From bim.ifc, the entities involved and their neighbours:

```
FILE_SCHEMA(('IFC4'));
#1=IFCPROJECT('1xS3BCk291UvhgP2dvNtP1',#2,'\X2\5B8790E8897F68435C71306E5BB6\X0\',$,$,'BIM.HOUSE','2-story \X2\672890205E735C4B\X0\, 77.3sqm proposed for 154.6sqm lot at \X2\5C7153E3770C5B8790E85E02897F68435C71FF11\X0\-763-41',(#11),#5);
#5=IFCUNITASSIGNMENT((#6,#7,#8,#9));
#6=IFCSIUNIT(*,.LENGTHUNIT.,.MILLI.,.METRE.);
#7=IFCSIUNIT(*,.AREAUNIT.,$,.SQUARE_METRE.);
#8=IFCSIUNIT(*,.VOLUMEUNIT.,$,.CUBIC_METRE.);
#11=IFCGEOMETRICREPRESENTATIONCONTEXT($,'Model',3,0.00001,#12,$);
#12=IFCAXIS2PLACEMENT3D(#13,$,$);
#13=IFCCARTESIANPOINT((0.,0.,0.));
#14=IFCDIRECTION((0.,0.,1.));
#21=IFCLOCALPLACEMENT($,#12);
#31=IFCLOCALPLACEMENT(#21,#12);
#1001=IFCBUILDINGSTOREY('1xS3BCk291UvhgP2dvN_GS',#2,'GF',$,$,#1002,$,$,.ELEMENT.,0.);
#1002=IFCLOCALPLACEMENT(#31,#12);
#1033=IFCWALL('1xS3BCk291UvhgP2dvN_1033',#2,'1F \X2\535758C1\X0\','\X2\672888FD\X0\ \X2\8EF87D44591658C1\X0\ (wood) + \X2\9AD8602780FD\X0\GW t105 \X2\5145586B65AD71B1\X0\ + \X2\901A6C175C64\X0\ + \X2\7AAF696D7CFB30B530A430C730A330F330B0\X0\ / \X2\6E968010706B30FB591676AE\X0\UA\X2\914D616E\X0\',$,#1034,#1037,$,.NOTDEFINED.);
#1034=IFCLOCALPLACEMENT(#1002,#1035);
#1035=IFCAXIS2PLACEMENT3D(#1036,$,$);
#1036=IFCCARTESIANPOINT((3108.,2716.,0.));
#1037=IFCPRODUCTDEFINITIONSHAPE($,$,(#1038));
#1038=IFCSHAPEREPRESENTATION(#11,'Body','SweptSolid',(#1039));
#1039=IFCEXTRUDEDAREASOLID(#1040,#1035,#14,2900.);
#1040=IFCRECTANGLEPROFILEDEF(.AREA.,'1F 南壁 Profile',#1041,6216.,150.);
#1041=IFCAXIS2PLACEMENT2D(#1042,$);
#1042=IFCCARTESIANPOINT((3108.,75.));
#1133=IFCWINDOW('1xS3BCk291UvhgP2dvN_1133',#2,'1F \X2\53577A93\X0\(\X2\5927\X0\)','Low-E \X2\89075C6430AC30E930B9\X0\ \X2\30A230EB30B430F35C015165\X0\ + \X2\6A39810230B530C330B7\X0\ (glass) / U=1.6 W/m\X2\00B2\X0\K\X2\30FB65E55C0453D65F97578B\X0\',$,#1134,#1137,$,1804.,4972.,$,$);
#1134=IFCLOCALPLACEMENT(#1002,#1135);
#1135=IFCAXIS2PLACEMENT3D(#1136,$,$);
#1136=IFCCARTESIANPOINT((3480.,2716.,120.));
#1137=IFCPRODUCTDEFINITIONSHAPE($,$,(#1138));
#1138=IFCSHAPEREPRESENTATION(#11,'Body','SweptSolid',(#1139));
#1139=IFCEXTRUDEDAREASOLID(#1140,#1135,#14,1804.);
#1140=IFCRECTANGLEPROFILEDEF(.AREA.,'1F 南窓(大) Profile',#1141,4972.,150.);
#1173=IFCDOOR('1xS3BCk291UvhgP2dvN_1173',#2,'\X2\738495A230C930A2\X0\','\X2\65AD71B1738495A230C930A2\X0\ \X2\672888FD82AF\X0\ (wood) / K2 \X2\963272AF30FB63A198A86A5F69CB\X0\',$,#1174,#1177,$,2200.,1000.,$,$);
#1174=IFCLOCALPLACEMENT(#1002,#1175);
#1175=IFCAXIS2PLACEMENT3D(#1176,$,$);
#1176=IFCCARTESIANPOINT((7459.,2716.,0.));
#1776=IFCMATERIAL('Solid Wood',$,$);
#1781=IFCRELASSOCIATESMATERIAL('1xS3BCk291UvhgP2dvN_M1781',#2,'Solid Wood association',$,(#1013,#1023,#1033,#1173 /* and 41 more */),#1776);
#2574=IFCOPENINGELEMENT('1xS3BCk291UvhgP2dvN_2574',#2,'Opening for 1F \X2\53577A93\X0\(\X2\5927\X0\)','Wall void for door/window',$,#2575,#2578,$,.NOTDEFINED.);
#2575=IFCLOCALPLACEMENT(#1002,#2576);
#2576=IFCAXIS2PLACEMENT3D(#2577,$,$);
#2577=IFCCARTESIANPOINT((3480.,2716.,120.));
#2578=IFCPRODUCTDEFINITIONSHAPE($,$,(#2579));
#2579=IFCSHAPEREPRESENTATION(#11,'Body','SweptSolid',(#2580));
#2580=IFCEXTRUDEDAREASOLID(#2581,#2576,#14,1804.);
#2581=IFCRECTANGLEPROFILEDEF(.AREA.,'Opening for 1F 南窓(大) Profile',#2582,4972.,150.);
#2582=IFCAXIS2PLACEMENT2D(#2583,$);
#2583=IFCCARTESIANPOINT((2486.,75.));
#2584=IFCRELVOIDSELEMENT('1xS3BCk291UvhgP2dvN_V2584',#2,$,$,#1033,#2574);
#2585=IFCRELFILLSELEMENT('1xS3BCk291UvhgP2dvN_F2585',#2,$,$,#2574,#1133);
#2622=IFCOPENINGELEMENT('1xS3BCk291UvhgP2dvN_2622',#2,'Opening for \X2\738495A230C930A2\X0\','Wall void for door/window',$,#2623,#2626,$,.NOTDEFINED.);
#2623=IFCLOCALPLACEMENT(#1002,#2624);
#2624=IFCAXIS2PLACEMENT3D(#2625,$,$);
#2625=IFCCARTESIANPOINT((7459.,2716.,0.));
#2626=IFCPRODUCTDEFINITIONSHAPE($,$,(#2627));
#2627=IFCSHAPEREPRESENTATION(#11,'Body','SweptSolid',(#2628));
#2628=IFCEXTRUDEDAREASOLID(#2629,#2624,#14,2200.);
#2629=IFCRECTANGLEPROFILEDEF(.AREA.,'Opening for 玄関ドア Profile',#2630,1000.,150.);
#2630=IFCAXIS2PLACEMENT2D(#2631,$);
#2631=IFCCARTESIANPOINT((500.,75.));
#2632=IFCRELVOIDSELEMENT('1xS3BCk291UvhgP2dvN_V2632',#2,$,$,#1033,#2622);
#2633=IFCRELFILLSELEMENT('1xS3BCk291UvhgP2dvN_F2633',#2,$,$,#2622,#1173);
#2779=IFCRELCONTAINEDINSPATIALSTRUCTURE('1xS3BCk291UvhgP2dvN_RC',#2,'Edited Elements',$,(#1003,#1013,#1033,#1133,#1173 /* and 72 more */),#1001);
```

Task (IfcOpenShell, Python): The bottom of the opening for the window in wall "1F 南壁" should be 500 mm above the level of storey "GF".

```python
import numpy as np
import ifcopenshell
import ifcopenshell.api.geometry
import ifcopenshell.geom
import ifcopenshell.util.element
import ifcopenshell.util.placement
import ifcopenshell.util.shape
import ifcopenshell.util.unit

model = ifcopenshell.open("bim.ifc")
unit_scale = ifcopenshell.util.unit.calculate_unit_scale(model)

window = model.by_id(1133)
opening = window.FillsVoids[0].RelatingOpeningElement
storey = ifcopenshell.util.element.get_container(window, ifc_class="IfcBuildingStorey")
level = ifcopenshell.util.placement.get_local_placement(storey.ObjectPlacement)[2, 3]

# The opening's origin need not be at the sill, so measure its lowest point.
shape = ifcopenshell.geom.create_shape(ifcopenshell.geom.settings(), opening)
bottom = ifcopenshell.util.shape.get_shape_bottom_elevation(shape, shape.geometry) / unit_scale
dz = level + 500.0 - bottom

shift = np.array([0.0, 0.0, dz])
# The window is not placed relative to its opening, so move both.
for product in (opening, window):
    matrix = ifcopenshell.util.placement.get_local_placement(product.ObjectPlacement)
    matrix[:3, 3] += shift
    ifcopenshell.api.geometry.edit_object_placement(model, product=product, matrix=matrix, is_si=False)

print(f"moved by {dz * unit_scale:+.3f} m")

model.write("bim_rev.ifc")
```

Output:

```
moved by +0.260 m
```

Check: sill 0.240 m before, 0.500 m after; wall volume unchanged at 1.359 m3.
